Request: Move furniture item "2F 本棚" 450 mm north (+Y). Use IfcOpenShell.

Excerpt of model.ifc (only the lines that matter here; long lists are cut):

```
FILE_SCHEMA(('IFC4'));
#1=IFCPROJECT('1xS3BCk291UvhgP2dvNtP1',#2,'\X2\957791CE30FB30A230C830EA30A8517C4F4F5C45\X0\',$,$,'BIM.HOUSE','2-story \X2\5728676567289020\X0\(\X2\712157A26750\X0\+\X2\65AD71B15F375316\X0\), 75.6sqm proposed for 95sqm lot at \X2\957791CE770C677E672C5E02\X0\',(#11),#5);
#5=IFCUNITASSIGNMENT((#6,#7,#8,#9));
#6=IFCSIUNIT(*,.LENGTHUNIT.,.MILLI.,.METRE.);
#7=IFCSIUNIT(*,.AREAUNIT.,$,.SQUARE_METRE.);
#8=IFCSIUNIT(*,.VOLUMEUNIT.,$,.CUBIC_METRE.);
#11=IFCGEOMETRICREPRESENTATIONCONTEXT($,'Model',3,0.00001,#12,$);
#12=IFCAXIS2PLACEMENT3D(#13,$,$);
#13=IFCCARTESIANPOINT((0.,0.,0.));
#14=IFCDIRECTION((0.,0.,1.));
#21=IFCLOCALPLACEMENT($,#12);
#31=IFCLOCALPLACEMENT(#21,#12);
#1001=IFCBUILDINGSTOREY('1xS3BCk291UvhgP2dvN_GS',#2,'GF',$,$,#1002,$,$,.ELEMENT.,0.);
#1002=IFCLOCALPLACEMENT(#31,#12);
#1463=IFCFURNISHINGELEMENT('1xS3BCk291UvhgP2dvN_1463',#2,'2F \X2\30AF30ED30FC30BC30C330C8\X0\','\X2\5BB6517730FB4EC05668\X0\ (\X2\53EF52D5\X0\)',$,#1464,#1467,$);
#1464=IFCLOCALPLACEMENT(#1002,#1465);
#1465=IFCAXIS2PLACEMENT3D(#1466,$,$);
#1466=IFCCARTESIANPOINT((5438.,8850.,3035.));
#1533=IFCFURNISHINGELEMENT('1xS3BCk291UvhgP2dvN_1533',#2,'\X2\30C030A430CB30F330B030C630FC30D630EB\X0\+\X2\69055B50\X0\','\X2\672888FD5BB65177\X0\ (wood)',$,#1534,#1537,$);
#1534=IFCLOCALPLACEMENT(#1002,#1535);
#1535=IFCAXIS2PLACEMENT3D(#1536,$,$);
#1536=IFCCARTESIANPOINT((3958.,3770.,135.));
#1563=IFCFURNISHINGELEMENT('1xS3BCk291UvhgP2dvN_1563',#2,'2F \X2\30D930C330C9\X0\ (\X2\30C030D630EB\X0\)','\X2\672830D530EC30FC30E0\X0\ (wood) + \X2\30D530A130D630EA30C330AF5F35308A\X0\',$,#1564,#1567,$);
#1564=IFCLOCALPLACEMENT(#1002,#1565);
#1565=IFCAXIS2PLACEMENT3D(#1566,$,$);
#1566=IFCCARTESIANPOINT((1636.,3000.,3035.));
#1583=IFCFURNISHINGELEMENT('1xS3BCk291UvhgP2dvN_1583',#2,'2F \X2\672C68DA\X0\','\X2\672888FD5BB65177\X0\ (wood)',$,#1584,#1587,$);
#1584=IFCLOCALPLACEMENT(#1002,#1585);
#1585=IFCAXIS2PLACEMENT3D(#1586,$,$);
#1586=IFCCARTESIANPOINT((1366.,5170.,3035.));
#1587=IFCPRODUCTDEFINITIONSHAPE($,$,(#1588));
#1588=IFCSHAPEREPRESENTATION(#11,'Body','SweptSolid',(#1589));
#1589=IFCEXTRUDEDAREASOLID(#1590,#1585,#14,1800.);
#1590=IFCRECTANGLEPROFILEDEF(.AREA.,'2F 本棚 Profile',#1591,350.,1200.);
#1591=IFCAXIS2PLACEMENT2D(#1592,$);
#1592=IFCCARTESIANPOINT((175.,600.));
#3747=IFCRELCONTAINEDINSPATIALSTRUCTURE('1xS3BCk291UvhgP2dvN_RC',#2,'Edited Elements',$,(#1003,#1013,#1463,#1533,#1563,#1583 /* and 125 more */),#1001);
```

```python
import ifcopenshell
import ifcopenshell.api.geometry
import ifcopenshell.util.placement
import ifcopenshell.util.unit

model = ifcopenshell.open("model.ifc")
unit_scale = ifcopenshell.util.unit.calculate_unit_scale(model)

item = model.by_id(1583)
matrix = ifcopenshell.util.placement.get_local_placement(item.ObjectPlacement)
matrix[1, 3] += 0.45 / unit_scale
ifcopenshell.api.geometry.edit_object_placement(model, product=item, matrix=matrix, is_si=False)

print(ifcopenshell.util.placement.get_local_placement(item.ObjectPlacement).round(3) + 0.0)

model.write("model_updated.ifc")
```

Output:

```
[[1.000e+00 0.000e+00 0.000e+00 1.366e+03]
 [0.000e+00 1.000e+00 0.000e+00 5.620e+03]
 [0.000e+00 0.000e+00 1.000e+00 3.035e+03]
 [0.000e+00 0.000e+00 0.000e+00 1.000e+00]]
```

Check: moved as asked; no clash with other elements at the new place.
